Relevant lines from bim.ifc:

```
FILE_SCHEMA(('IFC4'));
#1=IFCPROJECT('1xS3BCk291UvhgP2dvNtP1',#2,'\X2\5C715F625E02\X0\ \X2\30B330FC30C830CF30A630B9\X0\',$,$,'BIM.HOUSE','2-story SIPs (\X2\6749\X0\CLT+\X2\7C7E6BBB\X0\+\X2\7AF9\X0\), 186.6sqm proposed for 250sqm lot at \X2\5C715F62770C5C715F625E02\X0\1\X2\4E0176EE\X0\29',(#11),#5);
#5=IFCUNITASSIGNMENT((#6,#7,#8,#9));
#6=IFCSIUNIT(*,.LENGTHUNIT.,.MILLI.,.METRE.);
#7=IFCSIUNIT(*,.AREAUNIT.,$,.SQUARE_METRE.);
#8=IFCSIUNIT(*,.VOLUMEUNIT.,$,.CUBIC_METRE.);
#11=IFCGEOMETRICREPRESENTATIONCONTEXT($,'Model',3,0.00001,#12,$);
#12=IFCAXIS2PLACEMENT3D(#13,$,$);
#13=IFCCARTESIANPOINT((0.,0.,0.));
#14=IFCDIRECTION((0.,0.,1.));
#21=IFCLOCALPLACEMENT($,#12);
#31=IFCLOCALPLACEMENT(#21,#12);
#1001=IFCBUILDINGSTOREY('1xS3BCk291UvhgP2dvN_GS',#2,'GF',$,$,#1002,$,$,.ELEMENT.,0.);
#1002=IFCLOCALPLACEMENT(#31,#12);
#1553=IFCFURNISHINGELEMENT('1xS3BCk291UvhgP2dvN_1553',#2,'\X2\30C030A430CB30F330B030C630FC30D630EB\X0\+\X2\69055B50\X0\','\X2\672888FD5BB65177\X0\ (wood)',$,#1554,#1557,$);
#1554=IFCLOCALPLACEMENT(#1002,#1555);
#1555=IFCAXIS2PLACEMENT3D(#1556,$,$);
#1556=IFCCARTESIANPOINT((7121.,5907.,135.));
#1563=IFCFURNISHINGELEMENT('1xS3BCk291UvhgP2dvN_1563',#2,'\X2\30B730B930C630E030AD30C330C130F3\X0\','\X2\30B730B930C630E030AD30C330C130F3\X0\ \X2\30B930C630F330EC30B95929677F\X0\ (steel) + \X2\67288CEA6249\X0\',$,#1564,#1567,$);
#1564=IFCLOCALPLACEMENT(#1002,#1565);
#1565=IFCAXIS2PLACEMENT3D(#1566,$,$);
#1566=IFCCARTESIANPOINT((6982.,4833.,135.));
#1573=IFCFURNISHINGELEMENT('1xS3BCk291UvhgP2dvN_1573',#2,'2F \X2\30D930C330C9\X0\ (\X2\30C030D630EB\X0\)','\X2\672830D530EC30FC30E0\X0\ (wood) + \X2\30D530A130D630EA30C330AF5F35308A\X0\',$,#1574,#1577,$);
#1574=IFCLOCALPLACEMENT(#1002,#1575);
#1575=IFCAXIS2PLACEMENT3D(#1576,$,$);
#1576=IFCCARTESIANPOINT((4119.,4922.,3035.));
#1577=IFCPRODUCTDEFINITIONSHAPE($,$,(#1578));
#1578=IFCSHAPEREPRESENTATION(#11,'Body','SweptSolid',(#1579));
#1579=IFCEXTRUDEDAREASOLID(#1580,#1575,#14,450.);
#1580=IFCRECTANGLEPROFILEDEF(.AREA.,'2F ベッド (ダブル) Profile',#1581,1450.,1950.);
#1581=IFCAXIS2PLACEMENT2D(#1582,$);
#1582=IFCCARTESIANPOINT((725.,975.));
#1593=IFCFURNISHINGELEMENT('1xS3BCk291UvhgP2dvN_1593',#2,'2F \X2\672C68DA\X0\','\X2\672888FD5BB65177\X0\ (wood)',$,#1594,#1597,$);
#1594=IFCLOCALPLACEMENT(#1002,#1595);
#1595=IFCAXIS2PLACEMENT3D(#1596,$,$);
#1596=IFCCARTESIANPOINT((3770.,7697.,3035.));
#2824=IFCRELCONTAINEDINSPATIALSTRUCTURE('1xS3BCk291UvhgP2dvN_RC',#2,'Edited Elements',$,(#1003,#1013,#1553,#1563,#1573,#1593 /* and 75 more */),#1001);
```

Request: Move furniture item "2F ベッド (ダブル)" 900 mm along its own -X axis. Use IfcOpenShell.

```python
import ifcopenshell
import ifcopenshell.api.geometry
import ifcopenshell.util.placement
import ifcopenshell.util.unit

model = ifcopenshell.open("bim.ifc")
unit_scale = ifcopenshell.util.unit.calculate_unit_scale(model)

item = model.by_id(1573)
matrix = ifcopenshell.util.placement.get_local_placement(item.ObjectPlacement)
matrix[:3, 3] -= matrix[:3, 0] * 0.9 / unit_scale
ifcopenshell.api.geometry.edit_object_placement(model, product=item, matrix=matrix, is_si=False)

print(ifcopenshell.util.placement.get_local_placement(item.ObjectPlacement).round(3) + 0.0)

model.write("bim_v2.ifc")
```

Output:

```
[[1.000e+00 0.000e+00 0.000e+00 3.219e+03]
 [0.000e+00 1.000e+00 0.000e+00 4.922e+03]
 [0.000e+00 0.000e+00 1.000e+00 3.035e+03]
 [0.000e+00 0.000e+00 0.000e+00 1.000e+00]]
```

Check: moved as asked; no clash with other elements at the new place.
